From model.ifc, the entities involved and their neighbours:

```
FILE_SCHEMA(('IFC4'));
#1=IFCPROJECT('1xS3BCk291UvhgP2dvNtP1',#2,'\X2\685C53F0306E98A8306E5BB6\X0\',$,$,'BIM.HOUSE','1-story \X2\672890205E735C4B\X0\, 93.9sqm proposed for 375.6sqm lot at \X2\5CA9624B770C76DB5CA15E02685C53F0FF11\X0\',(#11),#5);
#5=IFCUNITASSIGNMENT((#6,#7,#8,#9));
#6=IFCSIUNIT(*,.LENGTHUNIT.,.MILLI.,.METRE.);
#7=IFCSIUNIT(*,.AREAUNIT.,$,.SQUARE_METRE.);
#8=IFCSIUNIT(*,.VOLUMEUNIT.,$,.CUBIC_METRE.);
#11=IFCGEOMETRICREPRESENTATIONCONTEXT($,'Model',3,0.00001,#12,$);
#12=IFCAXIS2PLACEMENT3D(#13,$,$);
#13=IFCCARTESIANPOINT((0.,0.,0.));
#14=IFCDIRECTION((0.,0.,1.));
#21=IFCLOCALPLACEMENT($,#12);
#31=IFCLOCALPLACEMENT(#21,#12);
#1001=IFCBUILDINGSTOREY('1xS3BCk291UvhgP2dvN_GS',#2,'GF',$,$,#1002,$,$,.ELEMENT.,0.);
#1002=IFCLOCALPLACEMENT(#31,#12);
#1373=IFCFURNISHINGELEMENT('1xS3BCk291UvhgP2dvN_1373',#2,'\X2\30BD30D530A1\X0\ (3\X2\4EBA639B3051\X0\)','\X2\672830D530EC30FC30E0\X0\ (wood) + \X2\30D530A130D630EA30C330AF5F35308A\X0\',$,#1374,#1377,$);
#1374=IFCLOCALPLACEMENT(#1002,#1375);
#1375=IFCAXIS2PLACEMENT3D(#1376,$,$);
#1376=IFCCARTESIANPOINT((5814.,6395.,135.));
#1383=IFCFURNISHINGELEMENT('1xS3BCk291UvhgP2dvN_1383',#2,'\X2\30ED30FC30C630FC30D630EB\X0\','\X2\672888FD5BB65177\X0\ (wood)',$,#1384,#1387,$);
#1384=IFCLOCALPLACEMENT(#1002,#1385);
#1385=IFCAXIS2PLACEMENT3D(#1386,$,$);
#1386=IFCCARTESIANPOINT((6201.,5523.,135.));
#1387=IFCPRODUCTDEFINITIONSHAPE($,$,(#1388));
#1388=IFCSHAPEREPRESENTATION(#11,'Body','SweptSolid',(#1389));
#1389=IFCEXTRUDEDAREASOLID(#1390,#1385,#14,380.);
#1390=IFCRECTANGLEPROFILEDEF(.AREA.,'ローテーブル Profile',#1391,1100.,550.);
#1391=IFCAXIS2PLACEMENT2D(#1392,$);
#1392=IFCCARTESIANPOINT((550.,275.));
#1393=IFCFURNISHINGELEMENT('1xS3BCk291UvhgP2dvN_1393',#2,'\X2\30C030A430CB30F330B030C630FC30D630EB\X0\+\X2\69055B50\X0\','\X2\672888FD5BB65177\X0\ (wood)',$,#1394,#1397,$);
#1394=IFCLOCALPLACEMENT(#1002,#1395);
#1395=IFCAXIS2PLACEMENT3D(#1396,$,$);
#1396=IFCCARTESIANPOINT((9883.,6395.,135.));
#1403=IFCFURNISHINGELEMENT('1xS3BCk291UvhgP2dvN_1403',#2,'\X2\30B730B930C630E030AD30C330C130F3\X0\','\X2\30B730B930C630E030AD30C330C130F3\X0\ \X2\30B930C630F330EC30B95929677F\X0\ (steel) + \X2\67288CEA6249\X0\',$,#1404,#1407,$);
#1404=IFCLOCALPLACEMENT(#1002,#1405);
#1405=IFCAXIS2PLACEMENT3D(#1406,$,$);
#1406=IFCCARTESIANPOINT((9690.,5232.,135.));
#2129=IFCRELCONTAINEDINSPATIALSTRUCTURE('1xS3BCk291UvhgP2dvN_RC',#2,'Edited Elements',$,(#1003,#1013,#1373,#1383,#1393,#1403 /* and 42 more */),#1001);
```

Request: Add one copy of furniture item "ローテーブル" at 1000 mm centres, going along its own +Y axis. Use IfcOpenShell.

```python
import ifcopenshell
import ifcopenshell.api.geometry
import ifcopenshell.api.root
import ifcopenshell.util.element
import ifcopenshell.util.placement
import ifcopenshell.util.unit

model = ifcopenshell.open("model.ifc")
unit_scale = ifcopenshell.util.unit.calculate_unit_scale(model)


def reuse_history(source, copy):
    """copy_class also copies each property set's owner history, people and application; keep the originals."""
    for rel in copy.IsDefinedBy:
        if rel.is_a("IfcRelDefinesByProperties") and (history := rel.RelatingPropertyDefinition.OwnerHistory):
            rel.RelatingPropertyDefinition.OwnerHistory = source.OwnerHistory
            ifcopenshell.util.element.remove_deep2(model, history)


source = model.by_guid("1xS3BCk291UvhgP2dvN_1383")
base = ifcopenshell.util.placement.get_local_placement(source.ObjectPlacement)
step = base[:3, 1] * 1 / unit_scale

for i in range(1, 2):
    copy = ifcopenshell.api.root.copy_class(model, product=source)
    copy.Representation = ifcopenshell.util.element.copy_deep(
        model, source.Representation, exclude=["IfcGeometricRepresentationContext", "IfcRepresentationMap"]
    )
    reuse_history(source, copy)
    matrix = base.copy()
    matrix[:3, 3] += i * step
    print("added at", matrix[:3, 3].round(3) + 0.0)
    ifcopenshell.api.geometry.edit_object_placement(model, product=copy, matrix=matrix, is_si=False)

model.write("model_updated.ifc")
```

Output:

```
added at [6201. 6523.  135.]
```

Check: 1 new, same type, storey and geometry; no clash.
